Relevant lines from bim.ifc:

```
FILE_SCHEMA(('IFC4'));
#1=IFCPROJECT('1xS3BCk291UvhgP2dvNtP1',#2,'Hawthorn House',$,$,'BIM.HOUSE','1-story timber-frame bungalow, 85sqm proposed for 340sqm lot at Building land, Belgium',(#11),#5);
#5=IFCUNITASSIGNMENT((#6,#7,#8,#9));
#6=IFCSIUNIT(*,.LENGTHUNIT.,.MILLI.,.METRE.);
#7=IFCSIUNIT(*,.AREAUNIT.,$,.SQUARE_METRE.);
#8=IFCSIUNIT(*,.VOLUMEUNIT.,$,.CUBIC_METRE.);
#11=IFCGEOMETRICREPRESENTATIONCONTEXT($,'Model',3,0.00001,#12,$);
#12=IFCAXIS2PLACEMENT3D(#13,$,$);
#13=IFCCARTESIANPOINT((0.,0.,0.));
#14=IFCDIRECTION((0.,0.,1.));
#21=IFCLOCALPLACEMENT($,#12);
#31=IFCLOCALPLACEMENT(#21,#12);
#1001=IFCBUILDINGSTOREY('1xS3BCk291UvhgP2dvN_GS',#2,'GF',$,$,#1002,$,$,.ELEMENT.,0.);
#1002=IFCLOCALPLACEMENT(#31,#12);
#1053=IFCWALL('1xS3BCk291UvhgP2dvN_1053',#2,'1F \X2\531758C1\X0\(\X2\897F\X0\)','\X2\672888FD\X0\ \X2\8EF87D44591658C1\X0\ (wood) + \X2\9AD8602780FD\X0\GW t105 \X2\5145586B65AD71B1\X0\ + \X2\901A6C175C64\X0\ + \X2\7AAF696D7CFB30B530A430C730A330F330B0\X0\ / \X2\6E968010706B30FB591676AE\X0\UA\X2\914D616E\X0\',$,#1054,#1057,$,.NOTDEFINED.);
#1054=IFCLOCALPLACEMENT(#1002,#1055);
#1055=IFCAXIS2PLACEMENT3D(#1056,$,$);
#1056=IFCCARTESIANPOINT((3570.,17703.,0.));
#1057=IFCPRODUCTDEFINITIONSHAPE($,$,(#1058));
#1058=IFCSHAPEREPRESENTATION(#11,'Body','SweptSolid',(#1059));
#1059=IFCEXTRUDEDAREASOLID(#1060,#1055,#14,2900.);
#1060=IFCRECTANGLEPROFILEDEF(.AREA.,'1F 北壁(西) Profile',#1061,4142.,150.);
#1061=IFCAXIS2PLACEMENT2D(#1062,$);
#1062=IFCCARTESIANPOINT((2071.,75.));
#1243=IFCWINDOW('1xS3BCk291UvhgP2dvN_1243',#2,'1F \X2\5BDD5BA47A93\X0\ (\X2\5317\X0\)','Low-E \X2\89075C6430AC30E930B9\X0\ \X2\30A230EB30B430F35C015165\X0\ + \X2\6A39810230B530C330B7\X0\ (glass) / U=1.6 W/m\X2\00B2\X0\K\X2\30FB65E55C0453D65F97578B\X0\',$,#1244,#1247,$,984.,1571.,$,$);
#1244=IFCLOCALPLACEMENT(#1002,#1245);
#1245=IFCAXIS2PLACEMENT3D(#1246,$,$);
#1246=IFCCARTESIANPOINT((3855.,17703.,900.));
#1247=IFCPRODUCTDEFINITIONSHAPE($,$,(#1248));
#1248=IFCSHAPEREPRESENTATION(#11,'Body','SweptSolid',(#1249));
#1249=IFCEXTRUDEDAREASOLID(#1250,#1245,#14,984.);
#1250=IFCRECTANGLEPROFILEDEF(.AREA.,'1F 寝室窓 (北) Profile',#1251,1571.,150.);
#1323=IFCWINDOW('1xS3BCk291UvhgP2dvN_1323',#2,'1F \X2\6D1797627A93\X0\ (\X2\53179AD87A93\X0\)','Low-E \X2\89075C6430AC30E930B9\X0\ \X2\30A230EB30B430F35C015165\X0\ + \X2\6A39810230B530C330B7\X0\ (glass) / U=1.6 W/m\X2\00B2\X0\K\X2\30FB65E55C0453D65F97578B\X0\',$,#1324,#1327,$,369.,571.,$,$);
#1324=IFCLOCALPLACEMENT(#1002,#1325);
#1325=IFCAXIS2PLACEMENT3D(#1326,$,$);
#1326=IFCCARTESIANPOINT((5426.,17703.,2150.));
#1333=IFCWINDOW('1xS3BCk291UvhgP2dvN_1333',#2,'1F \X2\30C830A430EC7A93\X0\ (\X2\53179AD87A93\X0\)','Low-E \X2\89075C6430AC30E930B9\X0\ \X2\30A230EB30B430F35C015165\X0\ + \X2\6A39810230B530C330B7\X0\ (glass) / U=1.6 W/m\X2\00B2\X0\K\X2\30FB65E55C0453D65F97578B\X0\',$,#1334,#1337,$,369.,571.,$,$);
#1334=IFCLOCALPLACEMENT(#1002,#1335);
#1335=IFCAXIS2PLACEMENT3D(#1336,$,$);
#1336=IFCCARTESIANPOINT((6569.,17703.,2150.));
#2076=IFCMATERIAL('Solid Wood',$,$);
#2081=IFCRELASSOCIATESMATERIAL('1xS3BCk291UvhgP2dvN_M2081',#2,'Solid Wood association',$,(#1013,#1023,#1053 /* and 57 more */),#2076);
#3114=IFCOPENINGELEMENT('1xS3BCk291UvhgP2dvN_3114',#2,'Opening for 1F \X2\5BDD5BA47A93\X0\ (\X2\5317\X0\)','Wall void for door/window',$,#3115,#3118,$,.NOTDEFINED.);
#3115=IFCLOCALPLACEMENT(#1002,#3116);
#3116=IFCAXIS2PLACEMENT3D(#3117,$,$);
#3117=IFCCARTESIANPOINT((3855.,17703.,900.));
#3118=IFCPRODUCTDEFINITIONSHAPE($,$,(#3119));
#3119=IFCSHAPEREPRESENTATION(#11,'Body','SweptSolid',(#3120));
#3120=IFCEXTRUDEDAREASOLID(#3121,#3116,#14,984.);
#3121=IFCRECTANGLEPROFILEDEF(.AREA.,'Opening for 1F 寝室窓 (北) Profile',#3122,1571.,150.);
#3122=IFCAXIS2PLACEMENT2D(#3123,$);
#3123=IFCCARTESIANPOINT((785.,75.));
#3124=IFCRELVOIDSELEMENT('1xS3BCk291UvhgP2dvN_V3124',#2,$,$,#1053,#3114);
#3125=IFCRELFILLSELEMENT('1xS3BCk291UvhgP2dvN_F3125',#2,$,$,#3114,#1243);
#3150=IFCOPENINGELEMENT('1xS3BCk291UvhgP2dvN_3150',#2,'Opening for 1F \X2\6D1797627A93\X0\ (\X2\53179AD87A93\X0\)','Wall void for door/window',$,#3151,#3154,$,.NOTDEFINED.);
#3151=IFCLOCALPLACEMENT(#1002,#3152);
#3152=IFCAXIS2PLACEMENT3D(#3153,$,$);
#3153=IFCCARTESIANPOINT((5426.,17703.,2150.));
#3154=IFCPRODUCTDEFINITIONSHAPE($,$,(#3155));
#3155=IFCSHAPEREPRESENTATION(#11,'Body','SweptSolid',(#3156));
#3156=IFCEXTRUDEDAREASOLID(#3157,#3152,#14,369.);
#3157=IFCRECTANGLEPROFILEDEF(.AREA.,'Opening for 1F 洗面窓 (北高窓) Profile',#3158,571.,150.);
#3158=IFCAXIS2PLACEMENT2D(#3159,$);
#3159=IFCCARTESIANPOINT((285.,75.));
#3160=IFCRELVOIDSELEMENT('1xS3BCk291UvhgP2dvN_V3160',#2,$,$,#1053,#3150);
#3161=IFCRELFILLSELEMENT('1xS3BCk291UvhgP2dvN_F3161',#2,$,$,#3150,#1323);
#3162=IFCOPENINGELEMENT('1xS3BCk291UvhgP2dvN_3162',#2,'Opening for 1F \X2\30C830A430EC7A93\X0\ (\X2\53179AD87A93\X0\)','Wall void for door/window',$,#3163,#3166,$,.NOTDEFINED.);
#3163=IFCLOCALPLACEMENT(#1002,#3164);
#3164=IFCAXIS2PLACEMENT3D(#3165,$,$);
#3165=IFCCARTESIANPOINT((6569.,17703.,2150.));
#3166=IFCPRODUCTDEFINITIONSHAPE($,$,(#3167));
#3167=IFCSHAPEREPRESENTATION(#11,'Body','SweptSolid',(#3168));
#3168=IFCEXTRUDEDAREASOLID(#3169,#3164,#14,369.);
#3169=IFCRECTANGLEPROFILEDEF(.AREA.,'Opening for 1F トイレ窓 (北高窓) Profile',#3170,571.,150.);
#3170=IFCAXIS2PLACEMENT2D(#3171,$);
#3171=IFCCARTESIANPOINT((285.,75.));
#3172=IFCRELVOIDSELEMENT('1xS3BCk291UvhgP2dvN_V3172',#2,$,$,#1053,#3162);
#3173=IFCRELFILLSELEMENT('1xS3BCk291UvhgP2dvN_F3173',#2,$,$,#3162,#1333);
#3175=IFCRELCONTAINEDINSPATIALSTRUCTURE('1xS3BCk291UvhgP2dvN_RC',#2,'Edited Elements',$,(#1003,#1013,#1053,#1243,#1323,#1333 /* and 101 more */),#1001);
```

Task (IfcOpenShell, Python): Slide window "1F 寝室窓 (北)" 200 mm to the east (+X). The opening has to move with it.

```python
import ifcopenshell
import ifcopenshell.api.geometry
import ifcopenshell.util.placement

model = ifcopenshell.open("bim.ifc")

window = model.by_guid("1xS3BCk291UvhgP2dvN_1243")
opening = window.FillsVoids[0].RelatingOpeningElement
wall = opening.VoidsElements[0].RelatingBuildingElement

wall_matrix = ifcopenshell.util.placement.get_local_placement(wall.ObjectPlacement)
shift = wall_matrix[:3, 0] * 200.0
before = ifcopenshell.util.placement.get_local_placement(window.ObjectPlacement)[:3, 3].copy()

# The window is not placed relative to its opening, so move both.
for product in (opening, window):
    matrix = ifcopenshell.util.placement.get_local_placement(product.ObjectPlacement)
    matrix[:3, 3] += shift
    ifcopenshell.api.geometry.edit_object_placement(model, product=product, matrix=matrix, is_si=False)

after = ifcopenshell.util.placement.get_local_placement(window.ObjectPlacement)[:3, 3]
print("window moved by", (after - before).round(3) + 0.0)

model.write("bim-out.ifc")
```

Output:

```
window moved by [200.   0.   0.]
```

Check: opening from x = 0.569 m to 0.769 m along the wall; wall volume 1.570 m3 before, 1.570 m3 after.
